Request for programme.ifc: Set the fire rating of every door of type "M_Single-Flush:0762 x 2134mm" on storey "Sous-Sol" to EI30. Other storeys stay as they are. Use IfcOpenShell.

First a look at what the model holds.

```python
import ifcopenshell
import ifcopenshell.util.element

model = ifcopenshell.open("programme.ifc")
print(model.schema)
storey = next(s for s in model.by_type("IfcBuildingStorey") if s.Name == "Sous-Sol")
doors = [e for e in ifcopenshell.util.element.get_decomposition(storey) if e.is_a("IfcDoor")]
seen = {}
for e in doors:
    element_type = ifcopenshell.util.element.get_type(e)
    key = (element_type.Name if element_type != e and element_type else None, ifcopenshell.util.element.get_pset(e, "Pset_DoorCommon", "FireRating"))
    seen[key] = seen.get(key, 0) + 1
for (name, value), count in sorted(seen.items(), key=str):
    print(count, "x", name, "|", value)
```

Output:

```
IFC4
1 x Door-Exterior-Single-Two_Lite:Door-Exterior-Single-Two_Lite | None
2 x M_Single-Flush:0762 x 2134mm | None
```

```python
import ifcopenshell
import ifcopenshell.api.pset
import ifcopenshell.util.element

model = ifcopenshell.open("programme.ifc")

storey = next(s for s in model.by_type("IfcBuildingStorey") if s.Name == "Sous-Sol")
doors = [e for e in ifcopenshell.util.element.get_decomposition(storey) if e.is_a("IfcDoor")]

count = 0
for e in doors:
    element_type = ifcopenshell.util.element.get_type(e)
    if element_type in (None, e) or element_type.Name != "M_Single-Flush:0762 x 2134mm":
        continue
    # add_pset returns the element's existing set when there is one.
    pset = ifcopenshell.api.pset.add_pset(model, product=e, name="Pset_DoorCommon")
    ifcopenshell.api.pset.edit_pset(model, pset=pset, properties={"FireRating": "EI30"})
    count += 1

print(count, "doors updated")

model.write("programme_v2.ifc")
```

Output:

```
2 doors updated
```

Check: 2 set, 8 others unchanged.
